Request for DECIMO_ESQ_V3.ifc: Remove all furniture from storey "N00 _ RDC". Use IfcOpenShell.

First a look at what the model holds.

```python
import ifcopenshell
import ifcopenshell.util.element

model = ifcopenshell.open("DECIMO_ESQ_V3.ifc")
print(model.schema)
storey = next(s for s in model.by_type("IfcBuildingStorey") if s.Name == "N00 _ RDC")
furniture = [e for e in ifcopenshell.util.element.get_decomposition(storey) if e.is_a("IfcFurnishingElement")]
seen = {}
for e in furniture:
    element_type = ifcopenshell.util.element.get_type(e)
    name = element_type.Name if element_type not in (None, e) else None
    seen[name] = seen.get(name, 0) + 1
for name, count in sorted(seen.items(), key=str):
    print(count, "x", name)
```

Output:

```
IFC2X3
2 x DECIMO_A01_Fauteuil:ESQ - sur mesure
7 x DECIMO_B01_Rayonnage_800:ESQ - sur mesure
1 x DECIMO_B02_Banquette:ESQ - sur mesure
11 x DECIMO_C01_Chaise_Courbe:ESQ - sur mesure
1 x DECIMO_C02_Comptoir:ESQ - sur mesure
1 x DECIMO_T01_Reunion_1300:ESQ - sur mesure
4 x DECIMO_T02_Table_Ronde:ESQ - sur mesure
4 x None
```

```python
import ifcopenshell
import ifcopenshell.api.root
import ifcopenshell.util.element

model = ifcopenshell.open("DECIMO_ESQ_V3.ifc")

storey = next(s for s in model.by_type("IfcBuildingStorey") if s.Name == "N00 _ RDC")
furniture = [e for e in ifcopenshell.util.element.get_decomposition(storey) if e.is_a("IfcFurnishingElement")]

for e in furniture:
    ifcopenshell.api.root.remove_product(model, product=e)
print(len(furniture), "removed")

model.write("DECIMO_ESQ_V3_rev.ifc")
```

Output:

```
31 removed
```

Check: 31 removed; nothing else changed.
